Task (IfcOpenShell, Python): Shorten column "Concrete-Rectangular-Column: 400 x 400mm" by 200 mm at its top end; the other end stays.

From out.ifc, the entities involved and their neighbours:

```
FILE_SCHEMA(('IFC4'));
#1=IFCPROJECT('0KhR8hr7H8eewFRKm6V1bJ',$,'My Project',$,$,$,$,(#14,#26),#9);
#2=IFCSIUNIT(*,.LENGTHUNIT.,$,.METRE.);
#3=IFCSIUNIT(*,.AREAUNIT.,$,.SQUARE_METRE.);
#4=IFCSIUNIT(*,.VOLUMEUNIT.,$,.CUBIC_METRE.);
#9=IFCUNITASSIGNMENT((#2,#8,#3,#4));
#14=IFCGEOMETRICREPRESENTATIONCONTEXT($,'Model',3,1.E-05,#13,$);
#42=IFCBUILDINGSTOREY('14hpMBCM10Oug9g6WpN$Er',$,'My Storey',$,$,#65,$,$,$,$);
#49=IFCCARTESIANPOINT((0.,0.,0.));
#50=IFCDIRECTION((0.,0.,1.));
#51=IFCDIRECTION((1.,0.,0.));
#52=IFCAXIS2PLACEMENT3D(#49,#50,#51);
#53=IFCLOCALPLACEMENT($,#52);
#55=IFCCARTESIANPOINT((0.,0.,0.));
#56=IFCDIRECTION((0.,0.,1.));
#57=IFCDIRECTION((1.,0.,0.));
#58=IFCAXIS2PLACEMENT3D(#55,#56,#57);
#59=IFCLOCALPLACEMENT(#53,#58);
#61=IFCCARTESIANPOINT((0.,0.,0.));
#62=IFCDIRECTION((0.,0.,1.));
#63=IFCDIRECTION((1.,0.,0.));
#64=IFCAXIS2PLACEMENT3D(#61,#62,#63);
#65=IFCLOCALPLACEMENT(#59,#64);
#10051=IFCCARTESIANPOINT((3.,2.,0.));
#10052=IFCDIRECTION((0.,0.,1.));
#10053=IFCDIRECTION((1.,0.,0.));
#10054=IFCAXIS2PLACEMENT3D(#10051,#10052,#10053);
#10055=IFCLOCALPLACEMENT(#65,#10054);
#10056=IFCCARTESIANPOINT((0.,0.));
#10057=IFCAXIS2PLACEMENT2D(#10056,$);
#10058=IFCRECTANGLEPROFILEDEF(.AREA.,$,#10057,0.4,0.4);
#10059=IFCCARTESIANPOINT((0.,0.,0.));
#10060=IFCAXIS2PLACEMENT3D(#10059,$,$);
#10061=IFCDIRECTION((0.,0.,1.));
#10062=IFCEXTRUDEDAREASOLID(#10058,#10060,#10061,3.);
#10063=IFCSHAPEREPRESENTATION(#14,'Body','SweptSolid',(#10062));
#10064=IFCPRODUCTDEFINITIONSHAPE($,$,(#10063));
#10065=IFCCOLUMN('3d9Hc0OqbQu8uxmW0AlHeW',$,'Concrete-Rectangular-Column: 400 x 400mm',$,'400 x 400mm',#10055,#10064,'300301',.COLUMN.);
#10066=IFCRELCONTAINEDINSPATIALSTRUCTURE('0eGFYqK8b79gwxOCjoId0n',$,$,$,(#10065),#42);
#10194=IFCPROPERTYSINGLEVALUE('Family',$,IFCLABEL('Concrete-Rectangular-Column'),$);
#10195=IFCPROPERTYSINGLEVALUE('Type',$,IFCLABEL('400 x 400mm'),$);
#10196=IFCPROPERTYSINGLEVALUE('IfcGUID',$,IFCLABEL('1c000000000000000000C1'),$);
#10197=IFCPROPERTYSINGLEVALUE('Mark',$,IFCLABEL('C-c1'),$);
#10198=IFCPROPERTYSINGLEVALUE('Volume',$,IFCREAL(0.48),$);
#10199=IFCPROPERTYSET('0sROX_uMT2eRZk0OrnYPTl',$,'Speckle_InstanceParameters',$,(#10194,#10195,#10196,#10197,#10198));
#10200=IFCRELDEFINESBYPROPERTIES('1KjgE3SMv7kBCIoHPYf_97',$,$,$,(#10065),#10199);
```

```python
import ifcopenshell
import ifcopenshell.api.pset
import ifcopenshell.util.element

model = ifcopenshell.open("out.ifc")

member = model.by_guid("3d9Hc0OqbQu8uxmW0AlHeW")
change = -0.2

# The extrusion runs towards the end named, so only its depth changes.
body = next(r for r in member.Representation.Representations if r.RepresentationIdentifier == "Body")
solid = body.Items[0]
old_length = solid.Depth
solid.Depth += change

# Update the stored length and volume.
pset = model.by_id(ifcopenshell.util.element.get_pset(member, "Speckle_InstanceParameters", should_inherit=False)["id"])
ifcopenshell.api.pset.edit_pset(model, pset=pset, properties={
    "Volume": model.create_entity("IfcReal", ifcopenshell.util.element.get_pset(member, "Speckle_InstanceParameters", "Volume") * solid.Depth / old_length),
})

print(f"length {old_length:g} -> {solid.Depth:g}")

model.write("out-out.ifc")
```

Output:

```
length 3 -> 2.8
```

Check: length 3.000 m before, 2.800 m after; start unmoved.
